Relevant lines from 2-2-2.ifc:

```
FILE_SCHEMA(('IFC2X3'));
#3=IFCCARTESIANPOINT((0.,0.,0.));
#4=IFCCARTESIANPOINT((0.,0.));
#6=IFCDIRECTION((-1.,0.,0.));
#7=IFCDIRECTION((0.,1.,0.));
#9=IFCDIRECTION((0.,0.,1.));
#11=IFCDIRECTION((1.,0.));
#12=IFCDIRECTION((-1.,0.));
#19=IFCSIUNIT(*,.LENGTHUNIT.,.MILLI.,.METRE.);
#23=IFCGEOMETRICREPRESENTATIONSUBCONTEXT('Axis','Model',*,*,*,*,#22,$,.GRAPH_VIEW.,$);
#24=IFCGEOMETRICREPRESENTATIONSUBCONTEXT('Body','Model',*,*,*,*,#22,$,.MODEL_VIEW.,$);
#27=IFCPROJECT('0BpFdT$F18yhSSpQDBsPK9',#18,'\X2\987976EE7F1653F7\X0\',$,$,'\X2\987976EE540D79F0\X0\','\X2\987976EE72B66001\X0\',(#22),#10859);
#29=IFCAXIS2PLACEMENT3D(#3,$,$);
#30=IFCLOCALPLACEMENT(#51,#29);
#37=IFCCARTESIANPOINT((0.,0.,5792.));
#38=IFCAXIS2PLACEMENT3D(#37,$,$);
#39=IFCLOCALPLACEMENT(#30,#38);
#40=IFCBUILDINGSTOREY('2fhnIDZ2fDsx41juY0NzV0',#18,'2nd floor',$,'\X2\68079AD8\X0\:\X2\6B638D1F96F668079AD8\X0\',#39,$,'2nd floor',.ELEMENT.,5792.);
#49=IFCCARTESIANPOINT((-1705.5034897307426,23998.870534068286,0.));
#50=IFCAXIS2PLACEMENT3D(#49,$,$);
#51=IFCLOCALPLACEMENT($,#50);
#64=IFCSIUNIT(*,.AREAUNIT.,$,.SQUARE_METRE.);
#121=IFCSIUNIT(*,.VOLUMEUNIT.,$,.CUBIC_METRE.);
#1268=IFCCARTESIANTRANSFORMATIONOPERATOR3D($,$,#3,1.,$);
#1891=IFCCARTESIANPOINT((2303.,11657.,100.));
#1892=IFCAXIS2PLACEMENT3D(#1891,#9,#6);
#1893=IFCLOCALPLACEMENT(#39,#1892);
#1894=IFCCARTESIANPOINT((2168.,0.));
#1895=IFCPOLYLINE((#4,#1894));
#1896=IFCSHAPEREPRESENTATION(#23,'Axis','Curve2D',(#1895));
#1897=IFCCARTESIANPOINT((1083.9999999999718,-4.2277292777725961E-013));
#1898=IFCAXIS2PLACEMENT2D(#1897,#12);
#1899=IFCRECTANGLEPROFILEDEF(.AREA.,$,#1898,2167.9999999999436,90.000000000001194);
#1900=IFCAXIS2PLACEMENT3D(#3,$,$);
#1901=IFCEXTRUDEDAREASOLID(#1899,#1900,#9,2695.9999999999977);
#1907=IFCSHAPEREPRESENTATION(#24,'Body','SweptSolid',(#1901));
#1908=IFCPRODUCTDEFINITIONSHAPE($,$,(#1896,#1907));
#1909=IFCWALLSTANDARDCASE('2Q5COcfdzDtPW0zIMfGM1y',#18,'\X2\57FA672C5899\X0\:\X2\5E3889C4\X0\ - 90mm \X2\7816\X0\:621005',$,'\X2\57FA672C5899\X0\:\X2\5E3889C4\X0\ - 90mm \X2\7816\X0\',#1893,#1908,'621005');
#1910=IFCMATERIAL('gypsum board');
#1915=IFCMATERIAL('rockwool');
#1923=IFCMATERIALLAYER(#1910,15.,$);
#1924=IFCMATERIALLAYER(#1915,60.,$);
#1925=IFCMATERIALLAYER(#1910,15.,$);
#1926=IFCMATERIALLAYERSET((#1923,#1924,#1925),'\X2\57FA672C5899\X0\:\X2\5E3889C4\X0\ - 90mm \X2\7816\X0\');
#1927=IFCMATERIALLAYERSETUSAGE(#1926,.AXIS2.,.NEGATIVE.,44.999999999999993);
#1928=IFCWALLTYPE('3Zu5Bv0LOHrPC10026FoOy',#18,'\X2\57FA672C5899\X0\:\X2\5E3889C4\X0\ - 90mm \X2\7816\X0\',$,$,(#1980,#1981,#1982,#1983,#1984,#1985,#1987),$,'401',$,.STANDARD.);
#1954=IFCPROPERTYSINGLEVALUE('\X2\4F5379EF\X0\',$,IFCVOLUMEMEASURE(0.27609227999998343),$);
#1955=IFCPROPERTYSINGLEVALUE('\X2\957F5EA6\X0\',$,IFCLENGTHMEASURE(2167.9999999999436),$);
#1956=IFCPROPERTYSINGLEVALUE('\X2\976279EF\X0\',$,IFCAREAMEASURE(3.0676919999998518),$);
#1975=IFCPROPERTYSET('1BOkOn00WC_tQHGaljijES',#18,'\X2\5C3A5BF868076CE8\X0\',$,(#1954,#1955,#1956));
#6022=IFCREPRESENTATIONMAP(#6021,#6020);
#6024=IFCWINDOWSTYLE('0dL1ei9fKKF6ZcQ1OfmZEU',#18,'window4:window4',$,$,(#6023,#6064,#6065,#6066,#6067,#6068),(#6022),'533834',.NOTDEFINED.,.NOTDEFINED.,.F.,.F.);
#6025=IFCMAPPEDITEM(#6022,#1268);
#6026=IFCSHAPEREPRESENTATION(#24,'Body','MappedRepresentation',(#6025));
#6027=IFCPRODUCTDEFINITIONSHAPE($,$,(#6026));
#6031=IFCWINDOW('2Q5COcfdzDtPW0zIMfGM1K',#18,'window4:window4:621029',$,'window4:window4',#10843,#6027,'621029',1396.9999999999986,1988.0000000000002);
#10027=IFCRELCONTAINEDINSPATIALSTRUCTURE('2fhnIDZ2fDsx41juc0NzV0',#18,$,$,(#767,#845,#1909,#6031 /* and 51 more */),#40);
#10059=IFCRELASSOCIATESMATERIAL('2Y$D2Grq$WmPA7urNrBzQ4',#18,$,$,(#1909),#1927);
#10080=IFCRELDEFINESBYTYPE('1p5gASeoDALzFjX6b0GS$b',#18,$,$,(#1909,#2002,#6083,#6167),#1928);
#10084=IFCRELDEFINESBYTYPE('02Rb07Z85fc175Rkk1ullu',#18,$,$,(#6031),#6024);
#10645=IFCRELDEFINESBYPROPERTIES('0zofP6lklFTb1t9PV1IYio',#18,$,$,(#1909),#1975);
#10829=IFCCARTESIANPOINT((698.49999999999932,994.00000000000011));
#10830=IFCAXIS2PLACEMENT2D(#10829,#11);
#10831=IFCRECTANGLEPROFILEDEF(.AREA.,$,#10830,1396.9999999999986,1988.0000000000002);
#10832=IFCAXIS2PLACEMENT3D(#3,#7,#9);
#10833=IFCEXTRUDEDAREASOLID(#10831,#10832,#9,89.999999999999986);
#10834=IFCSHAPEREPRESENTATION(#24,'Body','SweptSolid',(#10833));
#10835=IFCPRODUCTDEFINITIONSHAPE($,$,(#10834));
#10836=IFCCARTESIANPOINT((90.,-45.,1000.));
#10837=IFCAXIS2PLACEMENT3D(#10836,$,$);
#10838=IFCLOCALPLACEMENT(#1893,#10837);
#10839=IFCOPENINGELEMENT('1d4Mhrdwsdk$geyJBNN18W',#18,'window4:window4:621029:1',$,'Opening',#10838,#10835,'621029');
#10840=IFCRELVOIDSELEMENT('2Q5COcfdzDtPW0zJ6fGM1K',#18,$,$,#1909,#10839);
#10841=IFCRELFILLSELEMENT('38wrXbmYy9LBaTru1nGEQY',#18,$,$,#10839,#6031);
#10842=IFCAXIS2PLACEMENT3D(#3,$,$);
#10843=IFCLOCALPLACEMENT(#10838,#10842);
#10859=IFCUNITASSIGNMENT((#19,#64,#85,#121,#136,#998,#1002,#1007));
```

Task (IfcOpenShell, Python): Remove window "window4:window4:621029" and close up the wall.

```python
import ifcopenshell
import ifcopenshell.api.feature
import ifcopenshell.api.pset
import ifcopenshell.api.root
import ifcopenshell.geom
import ifcopenshell.util.element
import ifcopenshell.util.shape
import ifcopenshell.util.unit

model = ifcopenshell.open("2-2-2.ifc")
area_scale = ifcopenshell.util.unit.calculate_unit_scale(model, "AREAUNIT")
volume_scale = ifcopenshell.util.unit.calculate_unit_scale(model, "VOLUMEUNIT")
settings = ifcopenshell.geom.settings()


def volume(element):
    """Net volume in cubic metres, openings subtracted."""
    shape = ifcopenshell.geom.create_shape(settings, element)
    return ifcopenshell.util.shape.get_volume(shape.geometry)


window = model.by_id(6031)
opening = window.FillsVoids[0].RelatingOpeningElement
wall = opening.VoidsElements[0].RelatingBuildingElement
before = volume(wall)

ifcopenshell.api.root.remove_product(model, product=window)
ifcopenshell.api.feature.remove_feature(model, feature=opening)

after = volume(wall)
thickness = 0.09  # wall thickness in metres

# Update the wall's stored quantities.
pset = model.by_id(ifcopenshell.util.element.get_pset(wall, "尺寸标注", should_inherit=False)["id"])
ifcopenshell.api.pset.edit_pset(model, pset=pset, properties={
    "体积": model.create_entity("IfcVolumeMeasure", after / volume_scale),
    "面积": model.create_entity("IfcAreaMeasure", after / thickness / area_scale),
})

print(f"wall volume {before:.3f} -> {after:.3f} m3")

model.write("2-2-2_updated.ifc")
```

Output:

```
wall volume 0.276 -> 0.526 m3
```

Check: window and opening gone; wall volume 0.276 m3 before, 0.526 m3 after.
